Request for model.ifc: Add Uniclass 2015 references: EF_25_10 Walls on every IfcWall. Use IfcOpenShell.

First a look at what the model holds.

```python
import ifcopenshell

model = ifcopenshell.open("model.ifc")
print(model.schema)
print("classifications:", [c.Name for c in model.by_type("IfcClassification")])
for ifc_class in ("IfcDoor", "IfcRoof", "IfcStair", "IfcWall", "IfcWindow"):
    print(ifc_class, len(model.by_type(ifc_class)))
```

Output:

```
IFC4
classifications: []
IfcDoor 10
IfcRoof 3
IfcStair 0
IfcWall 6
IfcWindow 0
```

```python
import ifcopenshell
import ifcopenshell.api.classification

model = ifcopenshell.open("model.ifc")

system = ifcopenshell.api.classification.add_classification(model, classification="Uniclass 2015")

codes = {
    "IfcWall": ("EF_25_10", "Walls"),
}
for ifc_class, (code, name) in codes.items():
    products = model.by_type(ifc_class)
    ifcopenshell.api.classification.add_reference(
        model, products=products, classification=system, identification=code, name=name
    )
    print(code, len(products))

model.write("model_edited.ifc")
```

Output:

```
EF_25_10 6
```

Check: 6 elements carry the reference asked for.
